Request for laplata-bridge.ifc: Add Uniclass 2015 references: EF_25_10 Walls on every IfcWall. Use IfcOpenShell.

First a look at what the model holds.

```python
import ifcopenshell

model = ifcopenshell.open("laplata-bridge.ifc")
print(model.schema)
print("classifications:", [c.Name for c in model.by_type("IfcClassification")])
for ifc_class in ("IfcDoor", "IfcRoof", "IfcStair", "IfcWall", "IfcWindow"):
    print(ifc_class, len(model.by_type(ifc_class)))
```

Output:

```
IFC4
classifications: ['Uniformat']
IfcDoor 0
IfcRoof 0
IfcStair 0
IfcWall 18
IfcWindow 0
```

```python
import ifcopenshell
import ifcopenshell.api.classification

model = ifcopenshell.open("laplata-bridge.ifc")

system = ifcopenshell.api.classification.add_classification(model, classification="Uniclass 2015")

codes = {
    "IfcWall": ("EF_25_10", "Walls"),
}
for ifc_class, (code, name) in codes.items():
    products = model.by_type(ifc_class)
    ifcopenshell.api.classification.add_reference(
        model, products=products, classification=system, identification=code, name=name
    )
    print(code, len(products))

model.write("laplata-bridge_edited.ifc")
```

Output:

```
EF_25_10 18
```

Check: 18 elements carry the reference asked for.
